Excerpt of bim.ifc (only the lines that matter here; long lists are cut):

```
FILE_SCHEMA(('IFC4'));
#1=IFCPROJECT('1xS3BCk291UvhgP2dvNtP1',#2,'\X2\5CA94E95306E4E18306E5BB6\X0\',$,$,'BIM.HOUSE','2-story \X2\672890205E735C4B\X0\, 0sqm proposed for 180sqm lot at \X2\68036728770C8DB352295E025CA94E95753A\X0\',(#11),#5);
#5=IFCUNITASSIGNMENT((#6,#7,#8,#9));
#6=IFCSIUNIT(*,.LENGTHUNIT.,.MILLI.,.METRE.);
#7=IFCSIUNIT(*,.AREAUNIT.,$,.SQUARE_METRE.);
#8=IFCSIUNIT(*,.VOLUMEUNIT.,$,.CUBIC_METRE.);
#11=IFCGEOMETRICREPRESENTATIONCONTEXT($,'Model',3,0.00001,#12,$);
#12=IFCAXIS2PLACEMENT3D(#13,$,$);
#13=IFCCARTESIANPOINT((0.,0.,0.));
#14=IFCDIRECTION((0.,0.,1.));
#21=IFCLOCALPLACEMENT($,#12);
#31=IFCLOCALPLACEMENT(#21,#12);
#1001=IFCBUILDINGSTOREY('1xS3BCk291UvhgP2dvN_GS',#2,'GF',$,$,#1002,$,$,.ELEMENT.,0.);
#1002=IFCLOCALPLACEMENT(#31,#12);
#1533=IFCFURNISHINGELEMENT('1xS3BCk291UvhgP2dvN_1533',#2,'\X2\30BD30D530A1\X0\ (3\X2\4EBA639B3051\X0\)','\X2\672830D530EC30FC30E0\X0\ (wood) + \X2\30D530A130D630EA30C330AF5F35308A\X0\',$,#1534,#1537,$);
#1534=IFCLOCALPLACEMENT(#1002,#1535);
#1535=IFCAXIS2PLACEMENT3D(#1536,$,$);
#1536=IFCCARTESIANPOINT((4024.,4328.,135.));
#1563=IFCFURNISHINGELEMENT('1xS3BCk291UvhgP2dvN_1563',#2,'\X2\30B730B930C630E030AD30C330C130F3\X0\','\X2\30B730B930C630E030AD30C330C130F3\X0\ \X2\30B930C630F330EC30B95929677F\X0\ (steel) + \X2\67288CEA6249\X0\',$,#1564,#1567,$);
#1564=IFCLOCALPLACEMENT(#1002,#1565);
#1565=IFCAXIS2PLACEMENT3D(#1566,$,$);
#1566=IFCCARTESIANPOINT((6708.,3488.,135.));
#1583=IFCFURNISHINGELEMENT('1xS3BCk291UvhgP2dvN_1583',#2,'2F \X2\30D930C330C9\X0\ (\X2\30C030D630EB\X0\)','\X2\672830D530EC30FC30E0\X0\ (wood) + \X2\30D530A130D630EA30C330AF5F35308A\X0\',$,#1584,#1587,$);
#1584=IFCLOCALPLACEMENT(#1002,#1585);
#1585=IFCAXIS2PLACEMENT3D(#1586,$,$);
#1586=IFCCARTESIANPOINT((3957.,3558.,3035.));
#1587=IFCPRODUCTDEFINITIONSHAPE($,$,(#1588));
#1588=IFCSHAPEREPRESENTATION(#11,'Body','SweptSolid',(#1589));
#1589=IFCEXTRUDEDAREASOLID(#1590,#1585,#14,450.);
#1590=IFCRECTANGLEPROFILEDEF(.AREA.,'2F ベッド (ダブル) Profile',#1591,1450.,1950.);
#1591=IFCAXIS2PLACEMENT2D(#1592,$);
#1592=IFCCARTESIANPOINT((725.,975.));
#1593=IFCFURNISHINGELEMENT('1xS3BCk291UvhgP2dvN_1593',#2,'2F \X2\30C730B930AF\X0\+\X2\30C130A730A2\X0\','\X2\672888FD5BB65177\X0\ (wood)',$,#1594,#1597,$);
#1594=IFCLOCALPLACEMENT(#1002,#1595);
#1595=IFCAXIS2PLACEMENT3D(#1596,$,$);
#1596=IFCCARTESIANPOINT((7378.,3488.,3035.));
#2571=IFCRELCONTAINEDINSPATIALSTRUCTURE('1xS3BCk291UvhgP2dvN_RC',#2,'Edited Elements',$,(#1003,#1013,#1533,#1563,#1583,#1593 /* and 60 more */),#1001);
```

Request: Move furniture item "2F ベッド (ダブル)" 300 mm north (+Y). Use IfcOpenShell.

```python
import ifcopenshell
import ifcopenshell.api.geometry
import ifcopenshell.util.placement

model = ifcopenshell.open("bim.ifc")

item = model.by_guid("1xS3BCk291UvhgP2dvN_1583")
matrix = ifcopenshell.util.placement.get_local_placement(item.ObjectPlacement)
matrix[1, 3] += 300.0
ifcopenshell.api.geometry.edit_object_placement(model, product=item, matrix=matrix, is_si=False)

print(ifcopenshell.util.placement.get_local_placement(item.ObjectPlacement).round(3) + 0.0)

model.write("bim_edited.ifc")
```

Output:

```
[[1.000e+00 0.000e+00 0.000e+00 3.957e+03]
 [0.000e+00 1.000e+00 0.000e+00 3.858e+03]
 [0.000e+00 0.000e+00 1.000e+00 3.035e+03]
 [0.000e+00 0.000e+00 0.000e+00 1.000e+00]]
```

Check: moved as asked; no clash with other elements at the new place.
